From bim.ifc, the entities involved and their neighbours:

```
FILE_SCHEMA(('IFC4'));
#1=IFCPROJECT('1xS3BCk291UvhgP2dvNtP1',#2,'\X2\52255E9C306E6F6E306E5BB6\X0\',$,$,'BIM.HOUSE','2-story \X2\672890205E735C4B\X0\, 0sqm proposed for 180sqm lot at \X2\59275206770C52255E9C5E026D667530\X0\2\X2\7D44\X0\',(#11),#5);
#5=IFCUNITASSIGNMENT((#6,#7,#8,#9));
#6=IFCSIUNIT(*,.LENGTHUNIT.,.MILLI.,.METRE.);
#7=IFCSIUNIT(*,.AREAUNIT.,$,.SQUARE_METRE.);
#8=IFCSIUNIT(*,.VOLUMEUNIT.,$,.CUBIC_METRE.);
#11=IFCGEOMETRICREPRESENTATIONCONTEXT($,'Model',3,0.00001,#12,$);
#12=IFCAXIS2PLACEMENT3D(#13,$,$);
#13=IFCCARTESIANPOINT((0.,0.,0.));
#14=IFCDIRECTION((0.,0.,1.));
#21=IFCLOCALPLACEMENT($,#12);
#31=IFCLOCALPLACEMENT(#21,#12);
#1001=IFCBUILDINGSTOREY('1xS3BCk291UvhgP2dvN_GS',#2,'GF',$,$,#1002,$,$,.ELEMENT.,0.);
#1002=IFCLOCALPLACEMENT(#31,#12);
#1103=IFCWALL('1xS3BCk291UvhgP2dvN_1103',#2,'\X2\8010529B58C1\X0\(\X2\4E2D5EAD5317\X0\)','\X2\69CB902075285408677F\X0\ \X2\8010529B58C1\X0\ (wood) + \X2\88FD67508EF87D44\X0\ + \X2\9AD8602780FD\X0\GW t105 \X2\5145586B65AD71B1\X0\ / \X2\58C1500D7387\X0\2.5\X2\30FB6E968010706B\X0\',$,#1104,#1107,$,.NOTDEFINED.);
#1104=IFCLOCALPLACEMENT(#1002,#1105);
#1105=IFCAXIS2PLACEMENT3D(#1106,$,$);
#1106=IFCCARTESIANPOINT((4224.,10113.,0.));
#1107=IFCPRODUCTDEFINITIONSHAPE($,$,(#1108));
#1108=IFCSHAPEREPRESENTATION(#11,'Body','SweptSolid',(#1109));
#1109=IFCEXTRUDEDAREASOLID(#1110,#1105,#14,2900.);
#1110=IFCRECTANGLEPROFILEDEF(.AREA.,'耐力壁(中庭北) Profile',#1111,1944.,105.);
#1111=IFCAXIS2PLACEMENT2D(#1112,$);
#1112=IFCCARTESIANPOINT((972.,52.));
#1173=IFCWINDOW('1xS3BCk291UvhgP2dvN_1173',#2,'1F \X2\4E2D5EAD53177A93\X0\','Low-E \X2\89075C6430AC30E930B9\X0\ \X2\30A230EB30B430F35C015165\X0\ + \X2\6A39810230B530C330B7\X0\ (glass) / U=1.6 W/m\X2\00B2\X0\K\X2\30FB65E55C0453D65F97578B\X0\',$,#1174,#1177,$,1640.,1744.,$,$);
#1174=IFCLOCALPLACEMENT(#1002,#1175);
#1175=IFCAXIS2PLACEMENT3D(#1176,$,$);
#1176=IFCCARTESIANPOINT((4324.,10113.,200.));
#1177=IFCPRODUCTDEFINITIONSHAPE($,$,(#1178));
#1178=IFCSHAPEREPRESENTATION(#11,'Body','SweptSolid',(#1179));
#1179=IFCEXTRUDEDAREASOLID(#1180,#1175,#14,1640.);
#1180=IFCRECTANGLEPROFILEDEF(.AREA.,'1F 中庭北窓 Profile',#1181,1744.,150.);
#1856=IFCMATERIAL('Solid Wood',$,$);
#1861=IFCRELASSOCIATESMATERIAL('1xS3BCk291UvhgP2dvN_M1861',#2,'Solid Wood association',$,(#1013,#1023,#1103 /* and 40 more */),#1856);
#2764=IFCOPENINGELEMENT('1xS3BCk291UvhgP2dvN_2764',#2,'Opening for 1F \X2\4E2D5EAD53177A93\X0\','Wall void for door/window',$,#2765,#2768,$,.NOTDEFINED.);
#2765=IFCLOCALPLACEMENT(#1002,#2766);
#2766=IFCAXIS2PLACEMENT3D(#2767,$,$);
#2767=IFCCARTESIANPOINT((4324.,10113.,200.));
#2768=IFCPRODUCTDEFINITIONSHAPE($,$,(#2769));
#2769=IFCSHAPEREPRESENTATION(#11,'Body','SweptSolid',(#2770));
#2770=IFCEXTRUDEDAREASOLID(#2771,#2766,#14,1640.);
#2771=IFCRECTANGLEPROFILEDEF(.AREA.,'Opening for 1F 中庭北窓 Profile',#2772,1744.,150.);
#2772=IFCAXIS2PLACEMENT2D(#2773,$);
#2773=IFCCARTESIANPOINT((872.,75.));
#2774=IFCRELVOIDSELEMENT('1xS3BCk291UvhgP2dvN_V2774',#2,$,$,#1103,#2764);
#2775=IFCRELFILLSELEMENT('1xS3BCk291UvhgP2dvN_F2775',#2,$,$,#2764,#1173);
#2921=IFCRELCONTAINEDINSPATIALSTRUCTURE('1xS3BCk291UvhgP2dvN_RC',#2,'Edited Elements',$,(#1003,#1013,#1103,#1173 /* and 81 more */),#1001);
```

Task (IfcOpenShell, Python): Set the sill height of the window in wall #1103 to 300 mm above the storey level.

```python
import numpy as np
import ifcopenshell
import ifcopenshell.api.geometry
import ifcopenshell.geom
import ifcopenshell.util.element
import ifcopenshell.util.placement
import ifcopenshell.util.shape
import ifcopenshell.util.unit

model = ifcopenshell.open("bim.ifc")
unit_scale = ifcopenshell.util.unit.calculate_unit_scale(model)

window = model.by_guid("1xS3BCk291UvhgP2dvN_1173")
opening = window.FillsVoids[0].RelatingOpeningElement
storey = ifcopenshell.util.element.get_container(window, ifc_class="IfcBuildingStorey")
level = ifcopenshell.util.placement.get_local_placement(storey.ObjectPlacement)[2, 3]

# The opening's origin need not be at the sill, so measure its lowest point.
shape = ifcopenshell.geom.create_shape(ifcopenshell.geom.settings(), opening)
bottom = ifcopenshell.util.shape.get_shape_bottom_elevation(shape, shape.geometry) / unit_scale
dz = level + 300.0 - bottom

shift = np.array([0.0, 0.0, dz])
# The window is not placed relative to its opening, so move both.
for product in (opening, window):
    matrix = ifcopenshell.util.placement.get_local_placement(product.ObjectPlacement)
    matrix[:3, 3] += shift
    ifcopenshell.api.geometry.edit_object_placement(model, product=product, matrix=matrix, is_si=False)

print(f"moved by {dz * unit_scale:+.3f} m")

model.write("bim-out.ifc")
```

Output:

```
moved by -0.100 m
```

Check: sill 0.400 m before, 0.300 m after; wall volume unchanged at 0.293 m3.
